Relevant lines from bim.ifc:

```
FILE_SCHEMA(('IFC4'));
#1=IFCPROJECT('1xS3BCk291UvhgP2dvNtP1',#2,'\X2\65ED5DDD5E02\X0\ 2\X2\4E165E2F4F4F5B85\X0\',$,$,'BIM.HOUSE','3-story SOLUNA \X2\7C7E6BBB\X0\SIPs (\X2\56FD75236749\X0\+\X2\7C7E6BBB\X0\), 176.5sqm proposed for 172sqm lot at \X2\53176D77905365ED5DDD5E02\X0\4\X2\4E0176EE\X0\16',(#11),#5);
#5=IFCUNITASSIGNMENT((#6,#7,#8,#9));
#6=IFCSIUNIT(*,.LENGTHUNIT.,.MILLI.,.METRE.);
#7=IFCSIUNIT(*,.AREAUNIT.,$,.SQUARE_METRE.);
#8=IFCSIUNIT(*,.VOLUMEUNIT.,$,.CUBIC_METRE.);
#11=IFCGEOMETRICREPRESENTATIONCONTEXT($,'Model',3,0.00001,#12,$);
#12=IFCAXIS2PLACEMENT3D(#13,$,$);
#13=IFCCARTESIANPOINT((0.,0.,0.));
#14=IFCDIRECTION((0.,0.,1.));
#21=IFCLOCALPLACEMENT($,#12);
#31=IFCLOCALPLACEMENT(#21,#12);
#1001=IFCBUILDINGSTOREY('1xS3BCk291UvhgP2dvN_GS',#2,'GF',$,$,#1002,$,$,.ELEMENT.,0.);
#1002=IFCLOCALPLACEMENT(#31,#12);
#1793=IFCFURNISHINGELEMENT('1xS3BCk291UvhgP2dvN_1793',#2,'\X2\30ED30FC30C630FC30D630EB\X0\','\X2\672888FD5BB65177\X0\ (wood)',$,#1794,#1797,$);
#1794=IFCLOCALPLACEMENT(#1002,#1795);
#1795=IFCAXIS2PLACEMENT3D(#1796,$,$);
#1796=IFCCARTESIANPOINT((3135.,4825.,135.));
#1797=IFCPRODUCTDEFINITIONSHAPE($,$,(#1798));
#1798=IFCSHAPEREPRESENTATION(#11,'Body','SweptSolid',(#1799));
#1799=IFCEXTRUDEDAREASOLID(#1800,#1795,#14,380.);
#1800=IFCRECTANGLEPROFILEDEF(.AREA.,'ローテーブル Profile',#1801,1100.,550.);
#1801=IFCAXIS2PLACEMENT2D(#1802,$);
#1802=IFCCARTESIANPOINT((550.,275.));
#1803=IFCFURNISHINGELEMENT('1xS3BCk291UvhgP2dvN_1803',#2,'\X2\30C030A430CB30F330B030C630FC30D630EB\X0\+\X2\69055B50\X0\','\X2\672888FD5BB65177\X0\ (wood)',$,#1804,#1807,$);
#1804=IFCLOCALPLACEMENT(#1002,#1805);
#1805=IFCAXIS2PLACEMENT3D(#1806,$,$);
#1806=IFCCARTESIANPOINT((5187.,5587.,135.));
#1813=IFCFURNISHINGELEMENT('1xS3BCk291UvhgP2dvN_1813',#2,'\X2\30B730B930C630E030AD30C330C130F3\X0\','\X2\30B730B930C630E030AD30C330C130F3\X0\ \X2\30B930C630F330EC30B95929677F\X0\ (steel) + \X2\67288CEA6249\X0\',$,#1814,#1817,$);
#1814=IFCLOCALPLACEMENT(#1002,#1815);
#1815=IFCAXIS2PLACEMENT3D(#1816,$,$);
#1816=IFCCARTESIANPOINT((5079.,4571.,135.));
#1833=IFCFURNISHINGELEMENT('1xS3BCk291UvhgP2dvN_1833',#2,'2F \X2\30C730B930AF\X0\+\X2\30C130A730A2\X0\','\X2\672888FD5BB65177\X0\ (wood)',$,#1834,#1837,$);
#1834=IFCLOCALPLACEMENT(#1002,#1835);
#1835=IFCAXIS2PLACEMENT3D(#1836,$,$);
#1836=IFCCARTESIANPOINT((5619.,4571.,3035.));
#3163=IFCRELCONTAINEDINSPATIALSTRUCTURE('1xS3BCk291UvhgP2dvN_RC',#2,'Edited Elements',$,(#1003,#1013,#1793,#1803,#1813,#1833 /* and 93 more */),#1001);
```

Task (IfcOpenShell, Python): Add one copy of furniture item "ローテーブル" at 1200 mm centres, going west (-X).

```python
import numpy as np
import ifcopenshell
import ifcopenshell.api.geometry
import ifcopenshell.api.root
import ifcopenshell.util.element
import ifcopenshell.util.placement

model = ifcopenshell.open("bim.ifc")


def reuse_history(source, copy):
    """copy_class also copies each property set's owner history, people and application; keep the originals."""
    for rel in copy.IsDefinedBy:
        if rel.is_a("IfcRelDefinesByProperties") and (history := rel.RelatingPropertyDefinition.OwnerHistory):
            rel.RelatingPropertyDefinition.OwnerHistory = source.OwnerHistory
            ifcopenshell.util.element.remove_deep2(model, history)


source = model.by_guid("1xS3BCk291UvhgP2dvN_1793")
base = ifcopenshell.util.placement.get_local_placement(source.ObjectPlacement)
step = np.array([-1.0, 0.0, 0.0]) * 1200.0

for i in range(1, 2):
    copy = ifcopenshell.api.root.copy_class(model, product=source)
    copy.Representation = ifcopenshell.util.element.copy_deep(
        model, source.Representation, exclude=["IfcGeometricRepresentationContext", "IfcRepresentationMap"]
    )
    reuse_history(source, copy)
    matrix = base.copy()
    matrix[:3, 3] += i * step
    print("added at", matrix[:3, 3].round(3) + 0.0)
    ifcopenshell.api.geometry.edit_object_placement(model, product=copy, matrix=matrix, is_si=False)

model.write("bim_rev.ifc")
```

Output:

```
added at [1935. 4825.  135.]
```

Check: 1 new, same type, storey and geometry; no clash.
